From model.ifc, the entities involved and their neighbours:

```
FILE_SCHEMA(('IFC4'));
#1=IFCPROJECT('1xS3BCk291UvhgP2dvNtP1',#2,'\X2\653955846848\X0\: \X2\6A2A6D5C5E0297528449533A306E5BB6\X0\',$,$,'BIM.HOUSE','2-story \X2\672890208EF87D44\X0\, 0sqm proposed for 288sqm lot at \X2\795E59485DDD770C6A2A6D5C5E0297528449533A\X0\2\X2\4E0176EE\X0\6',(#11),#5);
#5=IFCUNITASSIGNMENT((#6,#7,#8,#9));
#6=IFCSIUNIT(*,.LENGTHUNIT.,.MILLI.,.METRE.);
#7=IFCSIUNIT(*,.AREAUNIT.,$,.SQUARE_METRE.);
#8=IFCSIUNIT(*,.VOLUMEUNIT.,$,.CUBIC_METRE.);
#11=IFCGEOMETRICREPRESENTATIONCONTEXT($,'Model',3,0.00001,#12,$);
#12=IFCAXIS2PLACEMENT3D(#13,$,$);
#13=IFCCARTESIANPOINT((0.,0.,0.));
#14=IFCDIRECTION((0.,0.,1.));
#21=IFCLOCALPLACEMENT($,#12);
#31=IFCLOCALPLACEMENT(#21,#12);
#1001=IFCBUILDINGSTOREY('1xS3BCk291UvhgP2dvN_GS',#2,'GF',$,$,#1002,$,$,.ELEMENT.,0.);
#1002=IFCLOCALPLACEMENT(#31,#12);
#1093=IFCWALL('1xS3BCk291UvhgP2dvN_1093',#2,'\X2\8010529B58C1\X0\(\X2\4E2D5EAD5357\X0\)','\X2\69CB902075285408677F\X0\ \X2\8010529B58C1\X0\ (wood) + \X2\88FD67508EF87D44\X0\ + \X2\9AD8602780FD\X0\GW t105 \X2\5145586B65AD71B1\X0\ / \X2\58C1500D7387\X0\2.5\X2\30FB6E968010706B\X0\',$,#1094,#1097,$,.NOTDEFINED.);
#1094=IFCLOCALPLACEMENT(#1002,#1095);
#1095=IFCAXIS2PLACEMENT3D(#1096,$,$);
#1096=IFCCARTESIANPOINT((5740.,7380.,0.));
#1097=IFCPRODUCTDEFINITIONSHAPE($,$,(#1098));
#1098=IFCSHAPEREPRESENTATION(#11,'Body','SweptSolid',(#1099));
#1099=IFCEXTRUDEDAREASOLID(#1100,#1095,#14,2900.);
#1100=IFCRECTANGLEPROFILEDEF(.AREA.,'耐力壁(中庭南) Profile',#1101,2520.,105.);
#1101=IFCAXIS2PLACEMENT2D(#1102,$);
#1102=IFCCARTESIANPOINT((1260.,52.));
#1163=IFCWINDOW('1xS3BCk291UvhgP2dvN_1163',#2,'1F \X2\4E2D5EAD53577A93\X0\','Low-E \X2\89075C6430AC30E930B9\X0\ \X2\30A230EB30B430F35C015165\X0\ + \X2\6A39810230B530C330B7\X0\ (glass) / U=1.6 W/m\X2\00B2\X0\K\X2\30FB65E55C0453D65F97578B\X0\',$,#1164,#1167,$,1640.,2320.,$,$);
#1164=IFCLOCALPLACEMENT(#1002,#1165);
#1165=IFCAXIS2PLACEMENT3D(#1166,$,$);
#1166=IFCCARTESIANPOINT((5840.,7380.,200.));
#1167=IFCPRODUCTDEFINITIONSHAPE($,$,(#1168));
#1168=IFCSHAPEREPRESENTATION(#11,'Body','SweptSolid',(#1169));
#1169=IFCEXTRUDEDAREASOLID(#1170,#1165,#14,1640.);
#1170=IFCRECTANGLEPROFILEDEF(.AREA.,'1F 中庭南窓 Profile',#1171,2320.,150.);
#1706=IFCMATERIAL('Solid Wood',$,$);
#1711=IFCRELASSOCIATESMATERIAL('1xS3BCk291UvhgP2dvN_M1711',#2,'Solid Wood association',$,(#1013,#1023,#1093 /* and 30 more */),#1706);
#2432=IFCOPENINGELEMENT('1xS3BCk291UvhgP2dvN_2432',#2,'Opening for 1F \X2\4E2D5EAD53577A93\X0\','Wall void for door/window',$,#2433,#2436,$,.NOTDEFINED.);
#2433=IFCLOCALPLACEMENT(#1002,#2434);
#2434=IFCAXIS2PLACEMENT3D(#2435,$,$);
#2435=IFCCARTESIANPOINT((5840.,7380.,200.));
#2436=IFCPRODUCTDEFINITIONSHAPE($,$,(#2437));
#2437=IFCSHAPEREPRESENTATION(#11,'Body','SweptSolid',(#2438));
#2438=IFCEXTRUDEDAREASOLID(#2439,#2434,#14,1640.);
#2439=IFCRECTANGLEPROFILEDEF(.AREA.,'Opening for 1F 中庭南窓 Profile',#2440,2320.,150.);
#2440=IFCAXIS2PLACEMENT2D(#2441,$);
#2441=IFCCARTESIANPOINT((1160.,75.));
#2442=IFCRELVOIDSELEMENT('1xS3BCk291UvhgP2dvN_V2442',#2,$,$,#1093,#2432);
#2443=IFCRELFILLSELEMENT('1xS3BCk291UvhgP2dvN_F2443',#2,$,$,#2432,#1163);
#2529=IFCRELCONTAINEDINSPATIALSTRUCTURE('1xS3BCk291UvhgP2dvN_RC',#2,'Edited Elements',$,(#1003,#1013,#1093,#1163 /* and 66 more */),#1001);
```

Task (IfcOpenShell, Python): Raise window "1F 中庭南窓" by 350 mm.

```python
import numpy as np
import ifcopenshell
import ifcopenshell.api.geometry
import ifcopenshell.util.placement
import ifcopenshell.util.unit

model = ifcopenshell.open("model.ifc")
unit_scale = ifcopenshell.util.unit.calculate_unit_scale(model)

window = model.by_guid("1xS3BCk291UvhgP2dvN_1163")
opening = window.FillsVoids[0].RelatingOpeningElement
dz = 0.35 / unit_scale

shift = np.array([0.0, 0.0, dz])
# The window is not placed relative to its opening, so move both.
for product in (opening, window):
    matrix = ifcopenshell.util.placement.get_local_placement(product.ObjectPlacement)
    matrix[:3, 3] += shift
    ifcopenshell.api.geometry.edit_object_placement(model, product=product, matrix=matrix, is_si=False)

print(f"moved by {dz * unit_scale:+.3f} m")

model.write("model_rev.ifc")
```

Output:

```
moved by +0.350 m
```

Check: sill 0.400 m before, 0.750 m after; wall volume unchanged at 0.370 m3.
